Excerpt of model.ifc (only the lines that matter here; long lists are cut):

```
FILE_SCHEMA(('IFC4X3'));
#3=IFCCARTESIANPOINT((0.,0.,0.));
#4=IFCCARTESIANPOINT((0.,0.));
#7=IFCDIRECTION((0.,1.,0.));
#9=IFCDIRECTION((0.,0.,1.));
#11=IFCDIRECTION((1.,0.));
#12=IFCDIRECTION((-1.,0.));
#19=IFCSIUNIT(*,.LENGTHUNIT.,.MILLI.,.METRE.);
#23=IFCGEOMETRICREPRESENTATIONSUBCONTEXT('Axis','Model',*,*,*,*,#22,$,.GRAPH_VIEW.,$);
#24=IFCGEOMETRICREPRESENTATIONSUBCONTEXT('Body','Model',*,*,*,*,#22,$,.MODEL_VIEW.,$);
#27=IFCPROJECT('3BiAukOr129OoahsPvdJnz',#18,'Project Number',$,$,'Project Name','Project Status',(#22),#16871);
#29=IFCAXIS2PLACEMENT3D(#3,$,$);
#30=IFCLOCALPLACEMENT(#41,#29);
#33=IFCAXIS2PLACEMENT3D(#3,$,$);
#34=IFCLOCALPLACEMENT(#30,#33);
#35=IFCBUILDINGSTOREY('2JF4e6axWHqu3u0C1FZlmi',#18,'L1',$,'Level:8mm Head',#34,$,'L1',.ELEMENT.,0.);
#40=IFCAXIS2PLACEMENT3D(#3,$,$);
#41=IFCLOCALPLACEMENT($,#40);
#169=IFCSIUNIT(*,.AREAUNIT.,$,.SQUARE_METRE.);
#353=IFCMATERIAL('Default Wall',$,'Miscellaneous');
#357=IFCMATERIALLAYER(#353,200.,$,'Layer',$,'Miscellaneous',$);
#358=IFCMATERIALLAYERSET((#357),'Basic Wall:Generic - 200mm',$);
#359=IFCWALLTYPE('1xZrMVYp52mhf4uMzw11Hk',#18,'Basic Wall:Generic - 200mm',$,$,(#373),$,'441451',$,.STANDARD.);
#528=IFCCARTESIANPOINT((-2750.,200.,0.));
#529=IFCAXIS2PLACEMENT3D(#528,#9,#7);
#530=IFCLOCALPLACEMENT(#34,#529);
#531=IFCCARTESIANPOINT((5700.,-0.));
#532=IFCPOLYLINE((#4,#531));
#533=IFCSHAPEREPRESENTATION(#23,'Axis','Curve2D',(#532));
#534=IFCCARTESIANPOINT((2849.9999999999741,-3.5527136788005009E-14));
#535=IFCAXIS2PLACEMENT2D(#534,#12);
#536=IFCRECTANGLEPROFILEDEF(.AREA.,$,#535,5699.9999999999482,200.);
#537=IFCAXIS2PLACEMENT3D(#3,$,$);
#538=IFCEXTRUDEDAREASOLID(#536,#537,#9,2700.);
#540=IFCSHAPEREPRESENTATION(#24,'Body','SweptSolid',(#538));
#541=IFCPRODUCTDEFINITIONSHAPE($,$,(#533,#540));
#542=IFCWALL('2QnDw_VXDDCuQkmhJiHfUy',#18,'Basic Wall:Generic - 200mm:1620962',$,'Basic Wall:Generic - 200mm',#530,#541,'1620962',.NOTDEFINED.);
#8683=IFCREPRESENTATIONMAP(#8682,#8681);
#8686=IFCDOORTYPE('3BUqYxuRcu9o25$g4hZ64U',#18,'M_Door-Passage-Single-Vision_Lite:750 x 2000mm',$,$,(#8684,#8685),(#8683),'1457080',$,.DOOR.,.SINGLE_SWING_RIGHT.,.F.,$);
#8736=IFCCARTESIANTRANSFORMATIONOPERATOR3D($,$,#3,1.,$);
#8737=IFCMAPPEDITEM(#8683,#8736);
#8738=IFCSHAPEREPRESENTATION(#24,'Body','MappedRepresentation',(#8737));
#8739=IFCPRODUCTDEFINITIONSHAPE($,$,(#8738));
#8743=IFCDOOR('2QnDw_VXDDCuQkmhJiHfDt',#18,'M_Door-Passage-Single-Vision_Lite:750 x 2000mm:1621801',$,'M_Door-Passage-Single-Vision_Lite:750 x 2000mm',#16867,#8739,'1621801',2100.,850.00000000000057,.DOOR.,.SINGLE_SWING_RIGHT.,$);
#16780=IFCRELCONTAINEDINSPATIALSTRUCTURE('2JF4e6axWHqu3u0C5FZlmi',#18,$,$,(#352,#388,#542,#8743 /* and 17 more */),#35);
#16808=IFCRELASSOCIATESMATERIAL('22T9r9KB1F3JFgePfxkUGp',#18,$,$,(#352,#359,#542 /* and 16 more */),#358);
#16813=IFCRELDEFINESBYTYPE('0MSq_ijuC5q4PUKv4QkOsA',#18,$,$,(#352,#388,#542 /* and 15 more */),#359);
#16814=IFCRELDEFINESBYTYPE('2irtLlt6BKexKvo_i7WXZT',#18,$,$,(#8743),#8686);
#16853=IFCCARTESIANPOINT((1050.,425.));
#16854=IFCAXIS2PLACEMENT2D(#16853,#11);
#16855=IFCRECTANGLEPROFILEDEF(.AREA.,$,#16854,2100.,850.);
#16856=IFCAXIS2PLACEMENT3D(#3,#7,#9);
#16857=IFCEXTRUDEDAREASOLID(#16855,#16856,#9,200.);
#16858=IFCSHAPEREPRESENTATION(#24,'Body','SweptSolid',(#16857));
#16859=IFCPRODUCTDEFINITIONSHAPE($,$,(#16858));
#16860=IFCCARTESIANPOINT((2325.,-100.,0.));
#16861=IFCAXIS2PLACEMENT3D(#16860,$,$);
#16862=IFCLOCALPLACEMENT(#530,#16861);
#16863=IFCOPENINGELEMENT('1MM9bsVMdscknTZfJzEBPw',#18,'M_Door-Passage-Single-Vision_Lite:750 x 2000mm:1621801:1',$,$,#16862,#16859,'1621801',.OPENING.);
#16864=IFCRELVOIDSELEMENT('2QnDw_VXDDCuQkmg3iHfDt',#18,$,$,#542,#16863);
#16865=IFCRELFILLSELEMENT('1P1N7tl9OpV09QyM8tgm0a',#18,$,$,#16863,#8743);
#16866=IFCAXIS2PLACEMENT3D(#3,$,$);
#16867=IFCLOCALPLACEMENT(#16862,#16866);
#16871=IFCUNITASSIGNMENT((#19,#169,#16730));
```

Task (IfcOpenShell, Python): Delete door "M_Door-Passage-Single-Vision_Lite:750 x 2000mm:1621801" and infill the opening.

```python
import ifcopenshell
import ifcopenshell.api.feature
import ifcopenshell.api.root
import ifcopenshell.geom
import ifcopenshell.util.shape

model = ifcopenshell.open("model.ifc")
settings = ifcopenshell.geom.settings()


def volume(element):
    """Net volume in cubic metres, openings subtracted."""
    shape = ifcopenshell.geom.create_shape(settings, element)
    return ifcopenshell.util.shape.get_volume(shape.geometry)


door = model.by_guid("2QnDw_VXDDCuQkmhJiHfDt")
opening = door.FillsVoids[0].RelatingOpeningElement
wall = opening.VoidsElements[0].RelatingBuildingElement
before = volume(wall)

ifcopenshell.api.root.remove_product(model, product=door)
ifcopenshell.api.feature.remove_feature(model, feature=opening)

after = volume(wall)

print(f"wall volume {before:.3f} -> {after:.3f} m3")

model.write("model_rev.ifc")
```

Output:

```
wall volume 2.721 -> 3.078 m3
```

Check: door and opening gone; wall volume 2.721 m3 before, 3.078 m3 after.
